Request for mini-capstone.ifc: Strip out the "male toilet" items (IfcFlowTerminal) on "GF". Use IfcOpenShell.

First a look at what the model holds.

```python
import ifcopenshell
import ifcopenshell.util.element

model = ifcopenshell.open("mini-capstone.ifc")
print(model.schema)
storey = next(s for s in model.by_type("IfcBuildingStorey") if s.Name == "GF")
terminals = [e for e in ifcopenshell.util.element.get_decomposition(storey) if e.is_a("IfcFlowTerminal")]
seen = {}
for e in terminals:
    element_type = ifcopenshell.util.element.get_type(e)
    name = element_type.Name if element_type not in (None, e) else None
    seen[name] = seen.get(name, 0) + 1
for name, count in sorted(seen.items(), key=str):
    print(count, "x", name)
```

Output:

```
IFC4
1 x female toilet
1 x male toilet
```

```python
import ifcopenshell
import ifcopenshell.api.root
import ifcopenshell.util.element

model = ifcopenshell.open("mini-capstone.ifc")

storey = next(s for s in model.by_type("IfcBuildingStorey") if s.Name == "GF")
terminals = [e for e in ifcopenshell.util.element.get_decomposition(storey) if e.is_a("IfcFlowTerminal")]
targets = [e for e in terminals if (t := ifcopenshell.util.element.get_type(e)) not in (None, e) and t.Name == "male toilet"]

for e in targets:
    ifcopenshell.api.root.remove_product(model, product=e)
print(len(targets), "removed")

model.write("mini-capstone_rev.ifc")
```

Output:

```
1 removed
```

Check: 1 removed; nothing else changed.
